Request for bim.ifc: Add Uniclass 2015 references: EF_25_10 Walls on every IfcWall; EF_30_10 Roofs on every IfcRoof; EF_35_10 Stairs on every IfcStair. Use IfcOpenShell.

First a look at what the model holds.

```python
import ifcopenshell

model = ifcopenshell.open("bim.ifc")
print(model.schema)
print("classifications:", [c.Name for c in model.by_type("IfcClassification")])
for ifc_class in ("IfcDoor", "IfcRoof", "IfcStair", "IfcWall", "IfcWindow"):
    print(ifc_class, len(model.by_type(ifc_class)))
```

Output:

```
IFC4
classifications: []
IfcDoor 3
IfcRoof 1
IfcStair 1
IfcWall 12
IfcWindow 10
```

```python
import ifcopenshell
import ifcopenshell.api.classification

model = ifcopenshell.open("bim.ifc")

system = ifcopenshell.api.classification.add_classification(model, classification="Uniclass 2015")

codes = {
    "IfcWall": ("EF_25_10", "Walls"),
    "IfcRoof": ("EF_30_10", "Roofs"),
    "IfcStair": ("EF_35_10", "Stairs"),
}
for ifc_class, (code, name) in codes.items():
    products = model.by_type(ifc_class)
    ifcopenshell.api.classification.add_reference(
        model, products=products, classification=system, identification=code, name=name
    )
    print(code, len(products))

model.write("bim_v2.ifc")
```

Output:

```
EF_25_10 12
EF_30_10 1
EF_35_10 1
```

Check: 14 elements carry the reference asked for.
